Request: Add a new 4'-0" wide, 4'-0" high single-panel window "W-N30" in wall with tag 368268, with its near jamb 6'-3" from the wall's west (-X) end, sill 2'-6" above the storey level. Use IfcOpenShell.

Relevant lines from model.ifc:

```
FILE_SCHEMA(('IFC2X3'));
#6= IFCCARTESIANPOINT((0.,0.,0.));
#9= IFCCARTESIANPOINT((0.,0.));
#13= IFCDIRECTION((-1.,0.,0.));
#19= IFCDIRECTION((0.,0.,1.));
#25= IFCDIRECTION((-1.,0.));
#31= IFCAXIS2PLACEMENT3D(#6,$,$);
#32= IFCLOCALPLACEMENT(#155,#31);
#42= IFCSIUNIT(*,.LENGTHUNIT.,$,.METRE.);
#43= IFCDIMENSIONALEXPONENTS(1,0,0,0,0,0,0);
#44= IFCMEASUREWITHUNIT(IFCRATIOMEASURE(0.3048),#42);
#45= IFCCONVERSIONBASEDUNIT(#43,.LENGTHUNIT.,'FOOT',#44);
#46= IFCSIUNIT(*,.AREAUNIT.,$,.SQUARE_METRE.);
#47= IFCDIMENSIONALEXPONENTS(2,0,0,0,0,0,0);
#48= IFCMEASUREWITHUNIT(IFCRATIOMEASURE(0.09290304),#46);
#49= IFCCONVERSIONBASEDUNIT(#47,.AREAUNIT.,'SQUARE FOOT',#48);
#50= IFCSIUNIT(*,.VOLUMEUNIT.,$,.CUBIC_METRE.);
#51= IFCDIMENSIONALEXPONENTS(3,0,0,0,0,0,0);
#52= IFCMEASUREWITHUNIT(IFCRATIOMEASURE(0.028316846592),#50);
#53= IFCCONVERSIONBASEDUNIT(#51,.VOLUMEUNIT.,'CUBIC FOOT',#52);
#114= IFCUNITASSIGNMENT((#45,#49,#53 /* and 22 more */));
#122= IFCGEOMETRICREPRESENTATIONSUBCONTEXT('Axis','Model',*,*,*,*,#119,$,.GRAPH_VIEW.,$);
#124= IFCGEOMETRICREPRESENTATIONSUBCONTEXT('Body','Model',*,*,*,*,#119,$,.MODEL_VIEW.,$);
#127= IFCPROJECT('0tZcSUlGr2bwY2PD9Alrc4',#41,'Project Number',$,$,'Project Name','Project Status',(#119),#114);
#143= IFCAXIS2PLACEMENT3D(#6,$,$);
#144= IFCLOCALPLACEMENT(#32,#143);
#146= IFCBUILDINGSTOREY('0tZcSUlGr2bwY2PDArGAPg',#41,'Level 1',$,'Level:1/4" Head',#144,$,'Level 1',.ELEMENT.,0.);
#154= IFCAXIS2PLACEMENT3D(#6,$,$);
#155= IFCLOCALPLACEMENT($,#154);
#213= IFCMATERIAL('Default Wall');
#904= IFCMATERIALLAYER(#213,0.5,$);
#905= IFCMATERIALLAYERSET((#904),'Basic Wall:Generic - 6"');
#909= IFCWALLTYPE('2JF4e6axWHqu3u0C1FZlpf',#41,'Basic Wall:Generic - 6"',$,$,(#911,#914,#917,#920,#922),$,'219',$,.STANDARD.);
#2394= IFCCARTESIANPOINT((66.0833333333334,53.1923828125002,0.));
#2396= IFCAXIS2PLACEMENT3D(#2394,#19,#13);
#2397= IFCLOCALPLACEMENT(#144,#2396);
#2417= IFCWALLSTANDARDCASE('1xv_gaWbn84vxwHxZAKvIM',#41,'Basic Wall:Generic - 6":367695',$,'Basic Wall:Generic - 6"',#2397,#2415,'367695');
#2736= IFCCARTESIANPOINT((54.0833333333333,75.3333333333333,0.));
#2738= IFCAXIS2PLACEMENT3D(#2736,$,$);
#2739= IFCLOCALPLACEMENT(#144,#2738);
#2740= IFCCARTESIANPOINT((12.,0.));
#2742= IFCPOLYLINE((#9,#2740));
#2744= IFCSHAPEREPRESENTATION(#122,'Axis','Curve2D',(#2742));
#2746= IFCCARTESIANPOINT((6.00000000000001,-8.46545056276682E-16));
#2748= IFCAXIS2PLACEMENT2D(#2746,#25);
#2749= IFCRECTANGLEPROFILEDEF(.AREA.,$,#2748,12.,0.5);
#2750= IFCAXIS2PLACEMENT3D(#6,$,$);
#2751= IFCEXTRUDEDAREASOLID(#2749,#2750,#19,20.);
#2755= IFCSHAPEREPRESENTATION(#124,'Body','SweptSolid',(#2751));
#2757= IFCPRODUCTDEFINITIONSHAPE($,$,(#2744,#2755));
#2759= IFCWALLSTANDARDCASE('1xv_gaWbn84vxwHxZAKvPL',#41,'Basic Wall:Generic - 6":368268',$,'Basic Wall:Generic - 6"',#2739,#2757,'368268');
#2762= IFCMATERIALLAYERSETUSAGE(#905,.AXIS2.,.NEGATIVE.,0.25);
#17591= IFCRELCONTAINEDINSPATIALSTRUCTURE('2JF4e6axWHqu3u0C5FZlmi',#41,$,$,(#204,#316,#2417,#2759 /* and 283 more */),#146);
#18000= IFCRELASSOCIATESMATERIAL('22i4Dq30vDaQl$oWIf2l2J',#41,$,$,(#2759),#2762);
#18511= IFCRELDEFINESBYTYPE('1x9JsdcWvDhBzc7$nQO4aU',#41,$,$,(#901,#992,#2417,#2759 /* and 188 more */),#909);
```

```python
import numpy as np
import ifcopenshell
import ifcopenshell.api.feature
import ifcopenshell.api.geometry
import ifcopenshell.api.root
import ifcopenshell.api.spatial
import ifcopenshell.api.type
import ifcopenshell.geom
import ifcopenshell.util.element
import ifcopenshell.util.placement
import ifcopenshell.util.representation
import ifcopenshell.util.shape
import ifcopenshell.util.unit

model = ifcopenshell.open("model.ifc")
unit_scale = ifcopenshell.util.unit.calculate_unit_scale(model)
settings = ifcopenshell.geom.settings()


def volume(element):
    """Net volume in cubic metres, openings subtracted."""
    shape = ifcopenshell.geom.create_shape(settings, element)
    return ifcopenshell.util.shape.get_volume(shape.geometry)


wall = model.by_guid("1xv_gaWbn84vxwHxZAKvPL")
storey = ifcopenshell.util.element.get_container(wall, ifc_class="IfcBuildingStorey")
context = ifcopenshell.util.representation.get_context(model, "Model", "Body", "MODEL_VIEW")
before = volume(wall)

width, height, from_end, sill = 1.2192, 1.2192, 1.905, 0.762  # metres

# The wall runs along its own X axis, and the end named is its -X end.
wall_shape = ifcopenshell.geom.create_shape(settings, wall)
x, y, z = ifcopenshell.util.shape.get_vertices(wall_shape.geometry).T
start = x.min() + from_end
face, thickness = float(y.min()), float(y.max() - y.min())
wall_matrix = ifcopenshell.util.placement.get_local_placement(wall.ObjectPlacement)
level = ifcopenshell.util.placement.get_local_placement(storey.ObjectPlacement)[2, 3]


def in_wall(x, y):
    """Placement at x, y metres in the wall's axes, at sill height."""
    matrix = wall_matrix.copy()
    matrix[:, 3] = wall_matrix @ np.array([x / unit_scale, y / unit_scale, 0.0, 1.0])
    matrix[2, 3] = level + sill / unit_scale
    return matrix


# Opening: a box that overshoots both wall faces by 50 mm.
opening = ifcopenshell.api.root.create_entity(model, ifc_class="IfcOpeningElement")
box = ifcopenshell.api.geometry.add_wall_representation(
    model, context=context, length=width, height=height, thickness=thickness + 0.1
)
ifcopenshell.api.geometry.assign_representation(model, product=opening, representation=box)
ifcopenshell.api.geometry.edit_object_placement(model, product=opening, matrix=in_wall(start, face - 0.05), is_si=False)
ifcopenshell.api.feature.add_feature(model, feature=opening, element=wall)

window = ifcopenshell.api.root.create_entity(model, ifc_class="IfcWindow", name="W-N30")
window.OverallWidth, window.OverallHeight = width / unit_scale, height / unit_scale
body = ifcopenshell.api.geometry.add_window_representation(
    model,
    context=context,
    overall_width=window.OverallWidth,
    overall_height=window.OverallHeight,
    partition_type="SINGLE_PANEL",
)
ifcopenshell.api.geometry.assign_representation(model, product=window, representation=body)
ifcopenshell.api.spatial.assign_container(model, products=[window], relating_structure=storey)
fills = ifcopenshell.api.feature.add_filling(model, opening=opening, element=window)
fills.OwnerHistory = window.OwnerHistory  # required in IFC2X3

# IFC2X3 keeps the operation on the window style.
style = ifcopenshell.api.root.create_entity(model, ifc_class="IfcWindowStyle", name="W-N30")
style.OperationType, style.ConstructionType = "SINGLE_PANEL", "NOTDEFINED"
style.ParameterTakesPrecedence = style.Sizeable = False
ifcopenshell.api.type.assign_type(model, related_objects=[window], relating_type=style)

# Centre the window in the wall's thickness.
ifcopenshell.api.geometry.edit_object_placement(model, product=window, matrix=in_wall(start, face), is_si=False)
window_shape = ifcopenshell.geom.create_shape(settings, window)
depth = ifcopenshell.util.shape.get_vertices(window_shape.geometry)[:, 1]
offset = face + thickness / 2 - (depth.min() + depth.max()) / 2
ifcopenshell.api.geometry.edit_object_placement(model, product=window, matrix=in_wall(start, offset), is_si=False)

after = volume(wall)

print(f"wall volume {before:.3f} -> {after:.3f} m3")

model.write("model_v2.ifc")
```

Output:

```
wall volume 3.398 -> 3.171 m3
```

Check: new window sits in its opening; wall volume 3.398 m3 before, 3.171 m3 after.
